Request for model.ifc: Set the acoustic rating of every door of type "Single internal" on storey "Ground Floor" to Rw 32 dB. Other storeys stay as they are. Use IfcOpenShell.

First a look at what the model holds.

```python
import ifcopenshell
import ifcopenshell.util.element

model = ifcopenshell.open("model.ifc")
print(model.schema)
storey = next(s for s in model.by_type("IfcBuildingStorey") if s.Name == "Ground Floor")
doors = [e for e in ifcopenshell.util.element.get_decomposition(storey) if e.is_a("IfcDoor")]
seen = {}
for e in doors:
    element_type = ifcopenshell.util.element.get_type(e)
    key = (element_type.Name if element_type != e and element_type else None, ifcopenshell.util.element.get_pset(e, "Pset_DoorCommon", "AcousticRating"))
    seen[key] = seen.get(key, 0) + 1
for (name, value), count in sorted(seen.items(), key=str):
    print(count, "x", name, "|", value)
```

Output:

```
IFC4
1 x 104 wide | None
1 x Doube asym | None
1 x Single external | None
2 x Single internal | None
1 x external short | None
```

```python
import ifcopenshell
import ifcopenshell.api.pset
import ifcopenshell.util.element

model = ifcopenshell.open("model.ifc")

storey = next(s for s in model.by_type("IfcBuildingStorey") if s.Name == "Ground Floor")
doors = [e for e in ifcopenshell.util.element.get_decomposition(storey) if e.is_a("IfcDoor")]

count = 0
for e in doors:
    element_type = ifcopenshell.util.element.get_type(e)
    if element_type in (None, e) or element_type.Name != "Single internal":
        continue
    # add_pset returns the element's existing set when there is one.
    pset = ifcopenshell.api.pset.add_pset(model, product=e, name="Pset_DoorCommon")
    ifcopenshell.api.pset.edit_pset(model, pset=pset, properties={"AcousticRating": "Rw 32 dB"})
    count += 1

print(count, "doors updated")

model.write("model_edited.ifc")
```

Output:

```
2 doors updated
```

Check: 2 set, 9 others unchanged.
